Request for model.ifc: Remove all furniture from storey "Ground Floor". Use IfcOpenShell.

First a look at what the model holds.

```python
import ifcopenshell
import ifcopenshell.util.element

model = ifcopenshell.open("model.ifc")
print(model.schema)
storey = next(s for s in model.by_type("IfcBuildingStorey") if s.Name == "Ground Floor")
furniture = [e for e in ifcopenshell.util.element.get_decomposition(storey) if e.is_a("IfcFurnishingElement")]
seen = {}
for e in furniture:
    element_type = ifcopenshell.util.element.get_type(e)
    name = element_type.Name if element_type not in (None, e) else None
    seen[name] = seen.get(name, 0) + 1
for name, count in sorted(seen.items(), key=str):
    print(count, "x", name)
```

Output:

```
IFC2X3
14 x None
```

```python
import ifcopenshell
import ifcopenshell.api.root
import ifcopenshell.util.element

model = ifcopenshell.open("model.ifc")

storey = next(s for s in model.by_type("IfcBuildingStorey") if s.Name == "Ground Floor")
furniture = [e for e in ifcopenshell.util.element.get_decomposition(storey) if e.is_a("IfcFurnishingElement")]

for e in furniture:
    ifcopenshell.api.root.remove_product(model, product=e)
print(len(furniture), "removed")

model.write("model_v2.ifc")
```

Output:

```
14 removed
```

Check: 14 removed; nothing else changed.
